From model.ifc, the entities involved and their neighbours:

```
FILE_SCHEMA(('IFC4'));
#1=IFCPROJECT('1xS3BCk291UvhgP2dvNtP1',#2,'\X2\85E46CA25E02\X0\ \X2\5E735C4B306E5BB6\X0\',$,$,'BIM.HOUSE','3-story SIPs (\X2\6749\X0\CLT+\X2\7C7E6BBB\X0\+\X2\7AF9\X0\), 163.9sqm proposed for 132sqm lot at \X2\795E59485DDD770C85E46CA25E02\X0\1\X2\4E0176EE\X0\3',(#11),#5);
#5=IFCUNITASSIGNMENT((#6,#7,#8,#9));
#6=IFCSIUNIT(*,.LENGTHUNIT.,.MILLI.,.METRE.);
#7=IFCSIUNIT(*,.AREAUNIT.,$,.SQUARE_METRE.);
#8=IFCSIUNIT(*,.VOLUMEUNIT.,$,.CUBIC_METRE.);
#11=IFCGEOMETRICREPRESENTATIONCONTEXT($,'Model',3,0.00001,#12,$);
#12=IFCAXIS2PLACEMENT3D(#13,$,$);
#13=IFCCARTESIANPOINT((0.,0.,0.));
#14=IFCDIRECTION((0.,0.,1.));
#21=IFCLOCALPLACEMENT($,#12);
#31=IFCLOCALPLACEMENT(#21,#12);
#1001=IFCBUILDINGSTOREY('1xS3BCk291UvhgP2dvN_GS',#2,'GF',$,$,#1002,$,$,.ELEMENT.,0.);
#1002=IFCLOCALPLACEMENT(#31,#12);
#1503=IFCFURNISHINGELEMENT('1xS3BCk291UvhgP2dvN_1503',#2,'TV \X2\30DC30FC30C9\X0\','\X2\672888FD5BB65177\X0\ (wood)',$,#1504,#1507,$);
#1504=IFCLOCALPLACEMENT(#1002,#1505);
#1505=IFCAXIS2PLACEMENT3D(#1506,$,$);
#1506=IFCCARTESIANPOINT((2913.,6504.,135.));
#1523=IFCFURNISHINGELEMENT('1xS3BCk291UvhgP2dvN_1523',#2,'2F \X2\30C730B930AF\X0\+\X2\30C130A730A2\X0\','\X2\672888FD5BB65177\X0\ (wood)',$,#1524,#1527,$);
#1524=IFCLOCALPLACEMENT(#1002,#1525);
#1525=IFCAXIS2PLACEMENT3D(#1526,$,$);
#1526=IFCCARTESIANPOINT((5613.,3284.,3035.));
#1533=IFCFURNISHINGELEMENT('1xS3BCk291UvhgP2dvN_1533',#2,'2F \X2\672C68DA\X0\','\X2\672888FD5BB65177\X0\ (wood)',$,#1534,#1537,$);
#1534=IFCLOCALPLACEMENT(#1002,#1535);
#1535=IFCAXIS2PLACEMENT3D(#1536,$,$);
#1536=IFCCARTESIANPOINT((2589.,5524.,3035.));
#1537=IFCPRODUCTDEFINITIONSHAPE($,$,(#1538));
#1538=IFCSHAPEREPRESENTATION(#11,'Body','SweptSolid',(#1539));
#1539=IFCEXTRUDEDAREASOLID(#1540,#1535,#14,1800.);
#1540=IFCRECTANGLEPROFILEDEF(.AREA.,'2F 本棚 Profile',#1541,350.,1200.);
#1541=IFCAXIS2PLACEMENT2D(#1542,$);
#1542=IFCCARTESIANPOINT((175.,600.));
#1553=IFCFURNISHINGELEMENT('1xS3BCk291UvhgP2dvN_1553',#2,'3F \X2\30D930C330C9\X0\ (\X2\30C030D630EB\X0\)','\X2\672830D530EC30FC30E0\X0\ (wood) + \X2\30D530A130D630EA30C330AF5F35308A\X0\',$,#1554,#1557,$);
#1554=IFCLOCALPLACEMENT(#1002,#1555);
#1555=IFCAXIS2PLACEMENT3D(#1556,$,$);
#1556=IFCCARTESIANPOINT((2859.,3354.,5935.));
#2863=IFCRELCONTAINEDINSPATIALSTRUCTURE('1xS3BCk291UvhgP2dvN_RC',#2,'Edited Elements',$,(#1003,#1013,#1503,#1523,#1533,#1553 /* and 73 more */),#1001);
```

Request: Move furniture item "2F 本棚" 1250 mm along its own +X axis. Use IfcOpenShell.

```python
import ifcopenshell
import ifcopenshell.api.geometry
import ifcopenshell.util.placement

model = ifcopenshell.open("model.ifc")

item = model.by_guid("1xS3BCk291UvhgP2dvN_1533")
matrix = ifcopenshell.util.placement.get_local_placement(item.ObjectPlacement)
matrix[:3, 3] += matrix[:3, 0] * 1250.0
ifcopenshell.api.geometry.edit_object_placement(model, product=item, matrix=matrix, is_si=False)

print(ifcopenshell.util.placement.get_local_placement(item.ObjectPlacement).round(3) + 0.0)

model.write("model_edited.ifc")
```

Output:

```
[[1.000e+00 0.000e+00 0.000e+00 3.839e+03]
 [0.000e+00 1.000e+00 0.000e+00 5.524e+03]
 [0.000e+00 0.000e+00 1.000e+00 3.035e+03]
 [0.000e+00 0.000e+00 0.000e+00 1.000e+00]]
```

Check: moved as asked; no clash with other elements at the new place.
